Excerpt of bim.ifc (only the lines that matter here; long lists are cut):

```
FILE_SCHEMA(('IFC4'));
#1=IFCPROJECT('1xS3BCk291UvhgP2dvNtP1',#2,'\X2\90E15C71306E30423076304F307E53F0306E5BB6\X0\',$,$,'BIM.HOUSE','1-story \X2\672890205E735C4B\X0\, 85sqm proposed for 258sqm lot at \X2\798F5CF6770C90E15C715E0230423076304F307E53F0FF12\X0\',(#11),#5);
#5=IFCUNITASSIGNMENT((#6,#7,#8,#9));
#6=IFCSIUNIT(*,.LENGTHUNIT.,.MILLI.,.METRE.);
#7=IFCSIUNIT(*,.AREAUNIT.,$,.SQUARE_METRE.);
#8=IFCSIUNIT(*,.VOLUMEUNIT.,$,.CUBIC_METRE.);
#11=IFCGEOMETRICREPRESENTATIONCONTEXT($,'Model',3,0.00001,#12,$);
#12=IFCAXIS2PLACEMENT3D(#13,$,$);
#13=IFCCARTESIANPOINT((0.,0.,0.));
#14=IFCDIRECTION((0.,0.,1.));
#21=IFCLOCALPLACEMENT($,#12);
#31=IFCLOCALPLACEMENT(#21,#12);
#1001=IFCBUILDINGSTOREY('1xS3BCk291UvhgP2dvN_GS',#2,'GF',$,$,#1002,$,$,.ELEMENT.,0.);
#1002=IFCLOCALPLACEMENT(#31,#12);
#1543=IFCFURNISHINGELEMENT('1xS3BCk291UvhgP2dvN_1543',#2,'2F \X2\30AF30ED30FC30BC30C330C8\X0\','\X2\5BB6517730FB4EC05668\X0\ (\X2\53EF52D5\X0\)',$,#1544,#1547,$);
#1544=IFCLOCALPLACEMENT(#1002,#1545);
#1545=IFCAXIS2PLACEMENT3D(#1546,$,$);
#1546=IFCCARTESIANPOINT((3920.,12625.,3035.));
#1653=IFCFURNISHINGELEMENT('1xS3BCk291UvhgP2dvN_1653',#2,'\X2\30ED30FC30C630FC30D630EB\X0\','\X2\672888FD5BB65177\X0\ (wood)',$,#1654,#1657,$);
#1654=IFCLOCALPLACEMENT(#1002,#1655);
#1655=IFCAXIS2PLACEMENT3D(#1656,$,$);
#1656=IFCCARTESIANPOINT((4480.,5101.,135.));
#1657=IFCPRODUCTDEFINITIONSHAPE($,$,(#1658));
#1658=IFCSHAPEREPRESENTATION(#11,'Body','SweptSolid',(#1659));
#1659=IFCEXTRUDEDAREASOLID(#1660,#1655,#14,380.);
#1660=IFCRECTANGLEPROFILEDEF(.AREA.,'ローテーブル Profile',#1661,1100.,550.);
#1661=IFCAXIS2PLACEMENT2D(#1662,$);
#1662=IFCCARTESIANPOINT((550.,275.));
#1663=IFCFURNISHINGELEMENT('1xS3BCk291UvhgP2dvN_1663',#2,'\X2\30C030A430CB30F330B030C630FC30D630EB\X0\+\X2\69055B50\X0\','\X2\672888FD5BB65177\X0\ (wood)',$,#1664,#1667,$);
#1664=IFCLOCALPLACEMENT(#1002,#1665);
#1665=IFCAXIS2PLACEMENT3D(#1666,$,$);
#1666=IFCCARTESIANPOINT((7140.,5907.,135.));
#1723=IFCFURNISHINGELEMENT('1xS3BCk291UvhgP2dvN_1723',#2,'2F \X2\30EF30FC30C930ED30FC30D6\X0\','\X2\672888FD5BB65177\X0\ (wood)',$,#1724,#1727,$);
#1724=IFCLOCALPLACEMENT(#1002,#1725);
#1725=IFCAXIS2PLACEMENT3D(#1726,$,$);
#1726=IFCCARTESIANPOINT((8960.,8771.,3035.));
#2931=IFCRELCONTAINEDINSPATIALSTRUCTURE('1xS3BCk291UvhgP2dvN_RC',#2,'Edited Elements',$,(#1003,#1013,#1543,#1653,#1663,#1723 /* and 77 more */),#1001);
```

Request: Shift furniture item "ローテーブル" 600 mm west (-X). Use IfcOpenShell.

```python
import ifcopenshell
import ifcopenshell.api.geometry
import ifcopenshell.util.placement

model = ifcopenshell.open("bim.ifc")

item = model.by_guid("1xS3BCk291UvhgP2dvN_1653")
matrix = ifcopenshell.util.placement.get_local_placement(item.ObjectPlacement)
matrix[0, 3] -= 600.0
ifcopenshell.api.geometry.edit_object_placement(model, product=item, matrix=matrix, is_si=False)

print(ifcopenshell.util.placement.get_local_placement(item.ObjectPlacement).round(3) + 0.0)

model.write("bim_v2.ifc")
```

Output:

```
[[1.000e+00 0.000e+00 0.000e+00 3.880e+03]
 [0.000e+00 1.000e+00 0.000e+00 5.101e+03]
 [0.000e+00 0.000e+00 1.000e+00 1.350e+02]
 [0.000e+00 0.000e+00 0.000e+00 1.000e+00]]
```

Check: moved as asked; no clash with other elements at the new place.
